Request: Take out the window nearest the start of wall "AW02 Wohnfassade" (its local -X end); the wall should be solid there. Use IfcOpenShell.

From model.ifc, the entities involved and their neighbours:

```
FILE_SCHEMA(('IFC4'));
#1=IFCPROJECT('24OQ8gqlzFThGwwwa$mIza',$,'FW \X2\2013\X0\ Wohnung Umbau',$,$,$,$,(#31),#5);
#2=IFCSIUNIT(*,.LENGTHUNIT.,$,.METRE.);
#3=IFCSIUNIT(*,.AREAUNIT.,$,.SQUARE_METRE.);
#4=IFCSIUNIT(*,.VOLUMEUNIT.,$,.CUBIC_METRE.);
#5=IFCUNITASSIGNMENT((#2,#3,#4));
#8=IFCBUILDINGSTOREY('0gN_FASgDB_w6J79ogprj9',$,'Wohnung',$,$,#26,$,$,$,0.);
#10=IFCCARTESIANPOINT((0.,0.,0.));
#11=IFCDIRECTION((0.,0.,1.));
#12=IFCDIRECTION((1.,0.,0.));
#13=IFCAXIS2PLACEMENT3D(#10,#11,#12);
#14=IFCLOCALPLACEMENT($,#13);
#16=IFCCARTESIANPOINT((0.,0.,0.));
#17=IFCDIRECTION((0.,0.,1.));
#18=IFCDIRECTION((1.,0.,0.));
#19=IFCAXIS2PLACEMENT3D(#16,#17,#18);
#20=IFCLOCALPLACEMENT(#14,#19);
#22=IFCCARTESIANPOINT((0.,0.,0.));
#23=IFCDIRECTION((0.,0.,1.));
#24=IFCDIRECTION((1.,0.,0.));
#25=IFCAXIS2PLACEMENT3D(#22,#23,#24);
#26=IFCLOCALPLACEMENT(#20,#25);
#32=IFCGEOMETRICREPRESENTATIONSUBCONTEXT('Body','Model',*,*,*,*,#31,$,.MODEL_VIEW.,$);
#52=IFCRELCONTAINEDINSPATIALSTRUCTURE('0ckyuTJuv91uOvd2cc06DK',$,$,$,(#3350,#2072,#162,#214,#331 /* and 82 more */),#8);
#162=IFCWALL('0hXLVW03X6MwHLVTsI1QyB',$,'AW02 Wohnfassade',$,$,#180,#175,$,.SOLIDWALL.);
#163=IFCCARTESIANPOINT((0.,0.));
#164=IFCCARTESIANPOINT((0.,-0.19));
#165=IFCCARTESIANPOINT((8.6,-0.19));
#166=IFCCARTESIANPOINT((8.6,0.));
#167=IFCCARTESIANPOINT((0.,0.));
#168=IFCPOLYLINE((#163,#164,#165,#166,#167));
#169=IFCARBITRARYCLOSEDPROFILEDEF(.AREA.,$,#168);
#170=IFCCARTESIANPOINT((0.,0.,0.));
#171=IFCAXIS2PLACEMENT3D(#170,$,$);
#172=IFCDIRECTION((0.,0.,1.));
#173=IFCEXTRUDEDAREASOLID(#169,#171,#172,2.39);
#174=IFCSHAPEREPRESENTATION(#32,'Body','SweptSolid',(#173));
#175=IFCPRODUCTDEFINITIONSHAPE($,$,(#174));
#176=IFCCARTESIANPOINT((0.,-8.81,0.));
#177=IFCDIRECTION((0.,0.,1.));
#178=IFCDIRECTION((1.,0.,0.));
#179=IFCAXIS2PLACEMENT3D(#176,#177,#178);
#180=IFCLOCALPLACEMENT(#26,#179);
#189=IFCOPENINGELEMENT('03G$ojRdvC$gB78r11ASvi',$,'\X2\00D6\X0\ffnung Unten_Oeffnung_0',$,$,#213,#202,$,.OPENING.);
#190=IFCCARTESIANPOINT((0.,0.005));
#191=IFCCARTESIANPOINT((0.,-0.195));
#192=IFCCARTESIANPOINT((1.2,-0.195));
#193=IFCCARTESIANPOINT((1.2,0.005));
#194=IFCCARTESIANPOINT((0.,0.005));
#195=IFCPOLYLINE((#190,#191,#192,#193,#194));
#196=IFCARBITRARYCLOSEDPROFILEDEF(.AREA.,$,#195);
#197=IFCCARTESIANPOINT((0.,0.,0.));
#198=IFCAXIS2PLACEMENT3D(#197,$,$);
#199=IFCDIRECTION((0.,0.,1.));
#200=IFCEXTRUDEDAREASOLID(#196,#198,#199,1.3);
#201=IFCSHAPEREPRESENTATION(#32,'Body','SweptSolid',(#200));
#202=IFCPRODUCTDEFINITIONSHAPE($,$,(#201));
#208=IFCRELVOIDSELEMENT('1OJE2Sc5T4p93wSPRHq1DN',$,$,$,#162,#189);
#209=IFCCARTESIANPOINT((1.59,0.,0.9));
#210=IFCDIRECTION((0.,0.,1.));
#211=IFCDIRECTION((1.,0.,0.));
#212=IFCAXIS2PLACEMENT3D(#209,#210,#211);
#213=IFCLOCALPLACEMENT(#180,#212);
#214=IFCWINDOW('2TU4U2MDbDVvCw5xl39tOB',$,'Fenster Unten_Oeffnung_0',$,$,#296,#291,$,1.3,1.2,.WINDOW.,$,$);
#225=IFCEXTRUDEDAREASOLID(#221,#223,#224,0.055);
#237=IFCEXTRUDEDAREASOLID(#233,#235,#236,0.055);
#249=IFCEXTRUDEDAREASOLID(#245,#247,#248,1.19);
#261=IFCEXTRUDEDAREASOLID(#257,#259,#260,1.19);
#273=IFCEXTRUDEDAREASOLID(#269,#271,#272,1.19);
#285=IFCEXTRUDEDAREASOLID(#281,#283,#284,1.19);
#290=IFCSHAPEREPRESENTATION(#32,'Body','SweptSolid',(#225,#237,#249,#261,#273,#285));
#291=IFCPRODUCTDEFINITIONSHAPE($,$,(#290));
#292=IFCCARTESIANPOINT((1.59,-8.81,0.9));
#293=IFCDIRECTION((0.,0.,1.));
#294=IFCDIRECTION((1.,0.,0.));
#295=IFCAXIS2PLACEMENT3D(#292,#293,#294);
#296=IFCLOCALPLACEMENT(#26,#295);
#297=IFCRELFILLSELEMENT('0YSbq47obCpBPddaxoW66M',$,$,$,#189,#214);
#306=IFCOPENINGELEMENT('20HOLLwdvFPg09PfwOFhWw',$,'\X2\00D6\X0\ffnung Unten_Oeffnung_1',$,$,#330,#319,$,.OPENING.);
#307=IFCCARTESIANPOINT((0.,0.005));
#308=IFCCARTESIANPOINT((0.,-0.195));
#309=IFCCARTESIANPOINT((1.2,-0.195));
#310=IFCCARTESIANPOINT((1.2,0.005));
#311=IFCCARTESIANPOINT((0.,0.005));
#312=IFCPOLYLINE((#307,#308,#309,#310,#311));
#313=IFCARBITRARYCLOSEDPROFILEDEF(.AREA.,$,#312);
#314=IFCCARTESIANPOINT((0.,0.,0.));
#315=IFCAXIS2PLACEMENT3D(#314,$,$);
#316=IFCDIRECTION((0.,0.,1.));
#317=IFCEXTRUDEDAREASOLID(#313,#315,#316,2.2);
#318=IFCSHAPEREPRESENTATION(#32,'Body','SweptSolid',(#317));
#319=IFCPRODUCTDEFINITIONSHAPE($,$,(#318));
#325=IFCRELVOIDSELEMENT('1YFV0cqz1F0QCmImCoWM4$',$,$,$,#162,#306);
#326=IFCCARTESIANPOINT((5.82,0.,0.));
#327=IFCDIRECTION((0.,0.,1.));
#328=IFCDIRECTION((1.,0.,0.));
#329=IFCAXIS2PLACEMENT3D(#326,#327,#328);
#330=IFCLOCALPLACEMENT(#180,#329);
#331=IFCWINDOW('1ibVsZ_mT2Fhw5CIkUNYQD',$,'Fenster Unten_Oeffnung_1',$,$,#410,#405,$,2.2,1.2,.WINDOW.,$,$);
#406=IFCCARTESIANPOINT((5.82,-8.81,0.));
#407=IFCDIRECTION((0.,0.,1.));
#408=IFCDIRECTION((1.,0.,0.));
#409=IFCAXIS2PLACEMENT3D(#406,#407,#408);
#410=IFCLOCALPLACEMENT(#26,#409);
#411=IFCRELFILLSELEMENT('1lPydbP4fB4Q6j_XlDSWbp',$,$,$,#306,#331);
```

```python
import ifcopenshell
import ifcopenshell.api.feature
import ifcopenshell.api.root
import ifcopenshell.geom
import ifcopenshell.util.shape

model = ifcopenshell.open("model.ifc")
settings = ifcopenshell.geom.settings()


def volume(element):
    """Net volume in cubic metres, openings subtracted."""
    shape = ifcopenshell.geom.create_shape(settings, element)
    return ifcopenshell.util.shape.get_volume(shape.geometry)


window = model.by_id(214)
opening = window.FillsVoids[0].RelatingOpeningElement
wall = opening.VoidsElements[0].RelatingBuildingElement
before = volume(wall)

ifcopenshell.api.root.remove_product(model, product=window)
ifcopenshell.api.feature.remove_feature(model, feature=opening)

after = volume(wall)

print(f"wall volume {before:.3f} -> {after:.3f} m3")

model.write("model_edited.ifc")
```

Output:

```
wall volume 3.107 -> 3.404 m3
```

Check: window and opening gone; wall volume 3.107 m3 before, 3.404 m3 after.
